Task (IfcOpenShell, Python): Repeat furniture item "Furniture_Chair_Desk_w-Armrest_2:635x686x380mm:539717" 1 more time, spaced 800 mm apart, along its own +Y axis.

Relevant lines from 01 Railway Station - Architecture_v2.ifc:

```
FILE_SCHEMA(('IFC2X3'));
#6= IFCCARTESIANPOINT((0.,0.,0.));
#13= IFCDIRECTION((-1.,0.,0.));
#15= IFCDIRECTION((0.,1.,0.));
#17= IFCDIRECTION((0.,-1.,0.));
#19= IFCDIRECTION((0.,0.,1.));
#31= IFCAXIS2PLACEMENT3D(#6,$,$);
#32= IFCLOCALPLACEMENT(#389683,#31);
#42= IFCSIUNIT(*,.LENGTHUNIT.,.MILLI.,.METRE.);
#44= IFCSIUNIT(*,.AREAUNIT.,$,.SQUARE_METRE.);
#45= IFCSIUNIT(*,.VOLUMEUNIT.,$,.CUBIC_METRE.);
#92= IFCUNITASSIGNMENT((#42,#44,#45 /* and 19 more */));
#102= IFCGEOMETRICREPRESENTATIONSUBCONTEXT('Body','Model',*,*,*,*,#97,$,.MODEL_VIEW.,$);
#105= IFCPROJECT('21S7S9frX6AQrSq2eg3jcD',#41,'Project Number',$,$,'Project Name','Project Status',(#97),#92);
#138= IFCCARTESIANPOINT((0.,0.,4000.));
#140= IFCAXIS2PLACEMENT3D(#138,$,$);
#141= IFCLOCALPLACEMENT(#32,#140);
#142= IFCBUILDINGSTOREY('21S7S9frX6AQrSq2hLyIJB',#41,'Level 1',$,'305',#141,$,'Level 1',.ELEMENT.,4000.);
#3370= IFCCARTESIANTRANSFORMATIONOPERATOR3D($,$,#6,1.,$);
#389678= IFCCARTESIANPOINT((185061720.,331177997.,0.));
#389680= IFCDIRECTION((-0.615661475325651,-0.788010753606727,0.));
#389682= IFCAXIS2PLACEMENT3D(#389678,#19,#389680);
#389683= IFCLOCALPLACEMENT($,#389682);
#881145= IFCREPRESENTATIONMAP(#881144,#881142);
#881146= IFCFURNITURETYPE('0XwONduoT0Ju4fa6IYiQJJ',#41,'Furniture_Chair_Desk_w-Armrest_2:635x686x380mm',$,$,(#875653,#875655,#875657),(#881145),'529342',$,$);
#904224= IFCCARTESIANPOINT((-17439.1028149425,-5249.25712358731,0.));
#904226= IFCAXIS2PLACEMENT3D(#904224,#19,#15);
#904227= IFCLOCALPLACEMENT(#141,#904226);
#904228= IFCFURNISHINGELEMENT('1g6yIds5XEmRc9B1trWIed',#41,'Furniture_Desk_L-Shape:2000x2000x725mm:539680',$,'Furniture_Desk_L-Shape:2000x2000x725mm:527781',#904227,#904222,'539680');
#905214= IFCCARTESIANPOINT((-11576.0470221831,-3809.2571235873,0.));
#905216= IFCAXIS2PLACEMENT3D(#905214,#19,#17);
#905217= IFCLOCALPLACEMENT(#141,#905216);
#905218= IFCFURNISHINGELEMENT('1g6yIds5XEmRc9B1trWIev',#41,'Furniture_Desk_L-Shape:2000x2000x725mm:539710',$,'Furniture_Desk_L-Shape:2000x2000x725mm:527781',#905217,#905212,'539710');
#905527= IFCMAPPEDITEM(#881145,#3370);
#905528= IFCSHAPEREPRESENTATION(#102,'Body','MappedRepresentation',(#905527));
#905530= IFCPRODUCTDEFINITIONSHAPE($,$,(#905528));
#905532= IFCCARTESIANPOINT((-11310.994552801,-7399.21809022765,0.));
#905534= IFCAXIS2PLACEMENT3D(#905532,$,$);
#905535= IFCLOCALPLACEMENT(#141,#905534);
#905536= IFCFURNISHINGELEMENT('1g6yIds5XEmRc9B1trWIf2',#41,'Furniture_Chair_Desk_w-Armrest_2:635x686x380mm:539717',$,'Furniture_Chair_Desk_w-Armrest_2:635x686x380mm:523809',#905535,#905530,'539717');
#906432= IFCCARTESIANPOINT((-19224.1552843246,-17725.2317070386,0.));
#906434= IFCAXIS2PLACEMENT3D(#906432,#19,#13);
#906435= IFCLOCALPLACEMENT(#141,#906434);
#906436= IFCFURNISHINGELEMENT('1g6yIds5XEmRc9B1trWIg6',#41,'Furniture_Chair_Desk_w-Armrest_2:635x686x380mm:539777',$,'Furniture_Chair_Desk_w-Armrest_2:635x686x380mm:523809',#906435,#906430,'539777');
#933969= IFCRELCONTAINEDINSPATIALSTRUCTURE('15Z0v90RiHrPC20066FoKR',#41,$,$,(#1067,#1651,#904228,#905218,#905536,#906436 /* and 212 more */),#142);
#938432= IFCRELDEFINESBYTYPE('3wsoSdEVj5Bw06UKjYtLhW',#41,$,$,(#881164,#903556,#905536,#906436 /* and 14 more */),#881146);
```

```python
import ifcopenshell
import ifcopenshell.api.geometry
import ifcopenshell.api.root
import ifcopenshell.util.element
import ifcopenshell.util.placement
import ifcopenshell.util.unit

model = ifcopenshell.open("01 Railway Station - Architecture_v2.ifc")
unit_scale = ifcopenshell.util.unit.calculate_unit_scale(model)


def reuse_history(source, copy):
    """copy_class also copies each property set's owner history, people and application; keep the originals."""
    for rel in copy.IsDefinedBy:
        if rel.is_a("IfcRelDefinesByProperties") and (history := rel.RelatingPropertyDefinition.OwnerHistory):
            rel.RelatingPropertyDefinition.OwnerHistory = source.OwnerHistory
            ifcopenshell.util.element.remove_deep2(model, history)


source = model.by_guid("1g6yIds5XEmRc9B1trWIf2")
base = ifcopenshell.util.placement.get_local_placement(source.ObjectPlacement)
step = base[:3, 1] * 0.8 / unit_scale

for i in range(1, 2):
    copy = ifcopenshell.api.root.copy_class(model, product=source)
    copy.Representation = ifcopenshell.util.element.copy_deep(
        model, source.Representation, exclude=["IfcGeometricRepresentationContext", "IfcRepresentationMap"]
    )
    copy.Name = "Furniture_Chair_Desk_w-Armrest_2:635x686x380mm"
    copy.Tag = None
    reuse_history(source, copy)
    matrix = base.copy()
    matrix[:3, 3] += i * step
    print("added at", matrix[:3, 3].round(3) + 0.0)
    ifcopenshell.api.geometry.edit_object_placement(model, product=copy, matrix=matrix, is_si=False)

model.write("01 Railway Station - Architecture_v2_rev.ifc")
```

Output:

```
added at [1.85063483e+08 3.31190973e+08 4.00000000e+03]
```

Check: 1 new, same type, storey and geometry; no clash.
